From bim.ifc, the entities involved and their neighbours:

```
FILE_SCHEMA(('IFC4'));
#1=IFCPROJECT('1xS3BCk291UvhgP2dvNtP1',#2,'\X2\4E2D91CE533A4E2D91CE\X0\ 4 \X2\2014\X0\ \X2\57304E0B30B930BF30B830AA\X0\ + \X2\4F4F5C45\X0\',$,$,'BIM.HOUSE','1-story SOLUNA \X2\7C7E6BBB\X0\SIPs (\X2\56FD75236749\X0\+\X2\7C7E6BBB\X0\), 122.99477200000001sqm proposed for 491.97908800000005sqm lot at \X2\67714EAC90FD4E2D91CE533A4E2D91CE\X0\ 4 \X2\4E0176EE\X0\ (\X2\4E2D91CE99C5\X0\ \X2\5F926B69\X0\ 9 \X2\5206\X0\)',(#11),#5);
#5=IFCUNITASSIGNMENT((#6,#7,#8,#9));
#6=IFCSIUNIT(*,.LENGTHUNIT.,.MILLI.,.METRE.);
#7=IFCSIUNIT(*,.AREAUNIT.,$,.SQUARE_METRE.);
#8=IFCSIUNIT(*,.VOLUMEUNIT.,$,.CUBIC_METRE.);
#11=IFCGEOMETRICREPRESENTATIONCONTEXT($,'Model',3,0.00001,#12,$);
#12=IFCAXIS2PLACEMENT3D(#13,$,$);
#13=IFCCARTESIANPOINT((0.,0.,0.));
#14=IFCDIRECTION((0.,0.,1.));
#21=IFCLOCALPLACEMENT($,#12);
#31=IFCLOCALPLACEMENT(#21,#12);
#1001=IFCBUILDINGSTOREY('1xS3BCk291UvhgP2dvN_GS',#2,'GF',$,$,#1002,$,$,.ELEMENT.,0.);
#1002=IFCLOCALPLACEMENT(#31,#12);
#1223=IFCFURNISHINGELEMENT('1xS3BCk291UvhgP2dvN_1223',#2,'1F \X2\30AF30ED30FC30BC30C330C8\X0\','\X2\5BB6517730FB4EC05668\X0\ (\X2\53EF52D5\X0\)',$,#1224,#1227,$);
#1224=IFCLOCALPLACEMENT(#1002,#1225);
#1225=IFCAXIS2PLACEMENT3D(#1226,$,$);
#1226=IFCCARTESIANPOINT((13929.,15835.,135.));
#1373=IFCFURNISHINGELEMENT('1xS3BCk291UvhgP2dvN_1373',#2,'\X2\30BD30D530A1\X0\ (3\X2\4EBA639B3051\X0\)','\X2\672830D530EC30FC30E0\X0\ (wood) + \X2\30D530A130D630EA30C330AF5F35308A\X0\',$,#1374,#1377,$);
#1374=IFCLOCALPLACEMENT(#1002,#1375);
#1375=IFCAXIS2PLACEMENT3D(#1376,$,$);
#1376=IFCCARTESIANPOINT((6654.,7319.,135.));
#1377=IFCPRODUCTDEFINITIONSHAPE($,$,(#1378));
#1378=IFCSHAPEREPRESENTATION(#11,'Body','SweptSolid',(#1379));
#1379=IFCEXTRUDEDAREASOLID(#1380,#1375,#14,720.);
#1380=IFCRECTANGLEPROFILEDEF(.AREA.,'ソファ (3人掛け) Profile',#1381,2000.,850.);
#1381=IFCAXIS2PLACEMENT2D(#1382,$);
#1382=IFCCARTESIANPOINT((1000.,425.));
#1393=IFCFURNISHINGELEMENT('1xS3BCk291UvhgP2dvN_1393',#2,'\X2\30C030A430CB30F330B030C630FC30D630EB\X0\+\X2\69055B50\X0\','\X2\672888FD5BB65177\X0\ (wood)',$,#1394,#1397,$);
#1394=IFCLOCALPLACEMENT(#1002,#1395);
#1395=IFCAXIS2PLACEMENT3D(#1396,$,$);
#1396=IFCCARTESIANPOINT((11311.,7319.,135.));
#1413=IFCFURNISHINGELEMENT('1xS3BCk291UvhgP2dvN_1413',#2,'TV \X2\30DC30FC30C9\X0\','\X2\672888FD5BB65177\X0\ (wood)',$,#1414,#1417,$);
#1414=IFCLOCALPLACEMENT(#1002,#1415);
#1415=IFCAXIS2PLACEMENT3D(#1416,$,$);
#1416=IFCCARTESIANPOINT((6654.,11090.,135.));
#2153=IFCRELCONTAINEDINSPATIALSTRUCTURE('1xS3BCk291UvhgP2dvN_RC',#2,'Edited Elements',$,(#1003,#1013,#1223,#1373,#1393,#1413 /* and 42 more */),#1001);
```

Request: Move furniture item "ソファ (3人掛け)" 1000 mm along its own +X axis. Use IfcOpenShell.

```python
import ifcopenshell
import ifcopenshell.api.geometry
import ifcopenshell.util.placement
import ifcopenshell.util.unit

model = ifcopenshell.open("bim.ifc")
unit_scale = ifcopenshell.util.unit.calculate_unit_scale(model)

item = model.by_id(1373)
matrix = ifcopenshell.util.placement.get_local_placement(item.ObjectPlacement)
matrix[:3, 3] += matrix[:3, 0] * 1 / unit_scale
ifcopenshell.api.geometry.edit_object_placement(model, product=item, matrix=matrix, is_si=False)

print(ifcopenshell.util.placement.get_local_placement(item.ObjectPlacement).round(3) + 0.0)

model.write("bim_edited.ifc")
```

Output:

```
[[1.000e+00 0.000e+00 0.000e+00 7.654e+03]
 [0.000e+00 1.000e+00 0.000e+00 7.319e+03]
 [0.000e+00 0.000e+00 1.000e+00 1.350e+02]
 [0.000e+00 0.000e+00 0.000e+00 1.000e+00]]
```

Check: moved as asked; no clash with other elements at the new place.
